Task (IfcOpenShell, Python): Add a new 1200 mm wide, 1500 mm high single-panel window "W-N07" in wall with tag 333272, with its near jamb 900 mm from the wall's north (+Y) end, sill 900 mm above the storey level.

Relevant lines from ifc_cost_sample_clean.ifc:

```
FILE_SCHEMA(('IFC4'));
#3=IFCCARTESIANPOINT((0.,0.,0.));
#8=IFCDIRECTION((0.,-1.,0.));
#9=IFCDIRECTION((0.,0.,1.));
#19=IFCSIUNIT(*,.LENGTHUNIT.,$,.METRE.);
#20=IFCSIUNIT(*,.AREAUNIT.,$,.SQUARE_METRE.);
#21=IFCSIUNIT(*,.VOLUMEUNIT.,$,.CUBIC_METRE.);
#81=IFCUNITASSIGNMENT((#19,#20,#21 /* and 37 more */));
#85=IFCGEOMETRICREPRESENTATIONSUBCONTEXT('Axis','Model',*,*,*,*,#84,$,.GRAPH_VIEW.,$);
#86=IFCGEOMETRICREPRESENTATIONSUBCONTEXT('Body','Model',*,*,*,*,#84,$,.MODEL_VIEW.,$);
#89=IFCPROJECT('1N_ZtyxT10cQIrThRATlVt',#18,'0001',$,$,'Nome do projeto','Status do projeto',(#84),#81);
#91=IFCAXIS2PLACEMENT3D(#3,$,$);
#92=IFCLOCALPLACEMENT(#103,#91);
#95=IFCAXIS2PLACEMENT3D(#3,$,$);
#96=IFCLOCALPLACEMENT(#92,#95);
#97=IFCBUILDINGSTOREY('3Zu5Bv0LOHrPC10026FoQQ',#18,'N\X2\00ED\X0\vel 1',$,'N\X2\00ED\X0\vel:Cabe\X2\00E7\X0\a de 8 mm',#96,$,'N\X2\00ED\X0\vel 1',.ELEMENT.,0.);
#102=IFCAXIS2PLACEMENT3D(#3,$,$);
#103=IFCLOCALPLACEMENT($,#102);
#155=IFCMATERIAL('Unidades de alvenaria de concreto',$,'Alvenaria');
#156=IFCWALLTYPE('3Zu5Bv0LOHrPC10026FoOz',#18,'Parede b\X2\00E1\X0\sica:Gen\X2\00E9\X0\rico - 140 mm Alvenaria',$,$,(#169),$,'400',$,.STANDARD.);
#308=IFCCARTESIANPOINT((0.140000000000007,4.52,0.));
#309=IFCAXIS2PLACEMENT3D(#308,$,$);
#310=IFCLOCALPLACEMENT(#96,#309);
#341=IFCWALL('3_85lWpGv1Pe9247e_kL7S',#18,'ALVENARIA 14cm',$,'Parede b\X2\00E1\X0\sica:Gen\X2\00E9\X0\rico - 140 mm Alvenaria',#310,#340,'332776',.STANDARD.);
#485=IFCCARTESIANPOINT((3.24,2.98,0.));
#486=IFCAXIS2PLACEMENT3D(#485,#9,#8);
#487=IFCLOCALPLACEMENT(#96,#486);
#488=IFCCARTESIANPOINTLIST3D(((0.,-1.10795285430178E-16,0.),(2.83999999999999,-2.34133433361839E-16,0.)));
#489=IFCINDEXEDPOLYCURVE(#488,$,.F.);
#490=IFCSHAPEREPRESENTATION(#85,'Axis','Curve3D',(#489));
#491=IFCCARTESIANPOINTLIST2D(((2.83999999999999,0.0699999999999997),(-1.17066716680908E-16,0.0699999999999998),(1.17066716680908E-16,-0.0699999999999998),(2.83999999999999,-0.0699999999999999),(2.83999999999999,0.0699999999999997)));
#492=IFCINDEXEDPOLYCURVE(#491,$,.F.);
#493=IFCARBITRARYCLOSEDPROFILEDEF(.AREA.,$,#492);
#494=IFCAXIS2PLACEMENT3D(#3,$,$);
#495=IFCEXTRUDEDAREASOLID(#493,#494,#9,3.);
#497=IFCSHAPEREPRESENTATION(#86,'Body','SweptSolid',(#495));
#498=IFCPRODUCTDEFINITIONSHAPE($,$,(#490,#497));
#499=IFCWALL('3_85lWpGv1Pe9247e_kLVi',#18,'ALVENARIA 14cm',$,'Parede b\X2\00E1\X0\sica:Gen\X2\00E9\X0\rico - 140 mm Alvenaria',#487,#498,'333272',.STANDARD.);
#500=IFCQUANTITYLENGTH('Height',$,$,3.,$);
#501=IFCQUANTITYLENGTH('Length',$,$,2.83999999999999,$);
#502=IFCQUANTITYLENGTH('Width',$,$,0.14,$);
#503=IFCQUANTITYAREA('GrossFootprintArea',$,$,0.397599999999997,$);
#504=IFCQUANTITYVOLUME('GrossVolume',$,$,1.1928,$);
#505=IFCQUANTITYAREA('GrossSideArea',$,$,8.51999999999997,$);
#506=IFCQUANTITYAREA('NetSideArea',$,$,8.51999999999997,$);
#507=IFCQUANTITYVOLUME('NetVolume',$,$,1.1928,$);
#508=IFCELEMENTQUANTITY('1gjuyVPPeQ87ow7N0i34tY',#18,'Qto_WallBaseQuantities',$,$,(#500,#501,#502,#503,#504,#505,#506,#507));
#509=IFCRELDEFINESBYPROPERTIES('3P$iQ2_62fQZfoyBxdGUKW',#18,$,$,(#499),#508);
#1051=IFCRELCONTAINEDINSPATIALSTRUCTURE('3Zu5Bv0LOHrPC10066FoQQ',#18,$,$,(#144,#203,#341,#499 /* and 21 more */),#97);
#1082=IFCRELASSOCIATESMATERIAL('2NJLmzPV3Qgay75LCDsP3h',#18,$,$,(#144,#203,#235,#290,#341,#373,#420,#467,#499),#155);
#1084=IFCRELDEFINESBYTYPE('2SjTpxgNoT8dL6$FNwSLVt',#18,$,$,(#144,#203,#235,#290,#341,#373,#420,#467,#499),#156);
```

```python
import numpy as np
import ifcopenshell
import ifcopenshell.api.feature
import ifcopenshell.api.geometry
import ifcopenshell.api.pset
import ifcopenshell.api.root
import ifcopenshell.api.spatial
import ifcopenshell.geom
import ifcopenshell.util.element
import ifcopenshell.util.placement
import ifcopenshell.util.representation
import ifcopenshell.util.shape
import ifcopenshell.util.unit

model = ifcopenshell.open("ifc_cost_sample_clean.ifc")
unit_scale = ifcopenshell.util.unit.calculate_unit_scale(model)
area_scale = ifcopenshell.util.unit.calculate_unit_scale(model, "AREAUNIT")
volume_scale = ifcopenshell.util.unit.calculate_unit_scale(model, "VOLUMEUNIT")
settings = ifcopenshell.geom.settings()


def volume(element):
    """Net volume in cubic metres, openings subtracted."""
    shape = ifcopenshell.geom.create_shape(settings, element)
    return ifcopenshell.util.shape.get_volume(shape.geometry)


wall = model.by_id(499)
storey = ifcopenshell.util.element.get_container(wall, ifc_class="IfcBuildingStorey")
context = ifcopenshell.util.representation.get_context(model, "Model", "Body", "MODEL_VIEW")
before = volume(wall)

width, height, from_end, sill = 1.2, 1.5, 0.9, 0.9  # metres

# The wall runs along its own X axis, and the end named is its -X end.
wall_shape = ifcopenshell.geom.create_shape(settings, wall)
x, y, z = ifcopenshell.util.shape.get_vertices(wall_shape.geometry).T
start = x.min() + from_end
face, thickness = float(y.min()), float(y.max() - y.min())
wall_matrix = ifcopenshell.util.placement.get_local_placement(wall.ObjectPlacement)
level = ifcopenshell.util.placement.get_local_placement(storey.ObjectPlacement)[2, 3]


def in_wall(x, y):
    """Placement at x, y metres in the wall's axes, at sill height."""
    matrix = wall_matrix.copy()
    matrix[:, 3] = wall_matrix @ np.array([x / unit_scale, y / unit_scale, 0.0, 1.0])
    matrix[2, 3] = level + sill / unit_scale
    return matrix


# Opening: a box that overshoots both wall faces by 50 mm.
opening = ifcopenshell.api.root.create_entity(model, ifc_class="IfcOpeningElement", predefined_type="OPENING")
box = ifcopenshell.api.geometry.add_wall_representation(
    model, context=context, length=width, height=height, thickness=thickness + 0.1
)
ifcopenshell.api.geometry.assign_representation(model, product=opening, representation=box)
ifcopenshell.api.geometry.edit_object_placement(model, product=opening, matrix=in_wall(start, face - 0.05), is_si=False)
ifcopenshell.api.feature.add_feature(model, feature=opening, element=wall)

window = ifcopenshell.api.root.create_entity(model, ifc_class="IfcWindow", name="W-N07", predefined_type="WINDOW")
window.OverallWidth, window.OverallHeight = width / unit_scale, height / unit_scale
window.PartitioningType = "SINGLE_PANEL"
body = ifcopenshell.api.geometry.add_window_representation(
    model,
    context=context,
    overall_width=window.OverallWidth,
    overall_height=window.OverallHeight,
    partition_type="SINGLE_PANEL",
)
ifcopenshell.api.geometry.assign_representation(model, product=window, representation=body)
ifcopenshell.api.spatial.assign_container(model, products=[window], relating_structure=storey)
ifcopenshell.api.feature.add_filling(model, opening=opening, element=window)

# Centre the window in the wall's thickness.
ifcopenshell.api.geometry.edit_object_placement(model, product=window, matrix=in_wall(start, face), is_si=False)
window_shape = ifcopenshell.geom.create_shape(settings, window)
depth = ifcopenshell.util.shape.get_vertices(window_shape.geometry)[:, 1]
offset = face + thickness / 2 - (depth.min() + depth.max()) / 2
ifcopenshell.api.geometry.edit_object_placement(model, product=window, matrix=in_wall(start, offset), is_si=False)

after = volume(wall)

# Update the wall's stored quantities.
qto = model.by_id(ifcopenshell.util.element.get_pset(wall, "Qto_WallBaseQuantities", should_inherit=False)["id"])
ifcopenshell.api.pset.edit_qto(model, qto=qto, properties={
    "NetSideArea": after / thickness / area_scale,
    "NetVolume": after / volume_scale,
})

print(f"wall volume {before:.3f} -> {after:.3f} m3")

model.write("ifc_cost_sample_clean_edited.ifc")
```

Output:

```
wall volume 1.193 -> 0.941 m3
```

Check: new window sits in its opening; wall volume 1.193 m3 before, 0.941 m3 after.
